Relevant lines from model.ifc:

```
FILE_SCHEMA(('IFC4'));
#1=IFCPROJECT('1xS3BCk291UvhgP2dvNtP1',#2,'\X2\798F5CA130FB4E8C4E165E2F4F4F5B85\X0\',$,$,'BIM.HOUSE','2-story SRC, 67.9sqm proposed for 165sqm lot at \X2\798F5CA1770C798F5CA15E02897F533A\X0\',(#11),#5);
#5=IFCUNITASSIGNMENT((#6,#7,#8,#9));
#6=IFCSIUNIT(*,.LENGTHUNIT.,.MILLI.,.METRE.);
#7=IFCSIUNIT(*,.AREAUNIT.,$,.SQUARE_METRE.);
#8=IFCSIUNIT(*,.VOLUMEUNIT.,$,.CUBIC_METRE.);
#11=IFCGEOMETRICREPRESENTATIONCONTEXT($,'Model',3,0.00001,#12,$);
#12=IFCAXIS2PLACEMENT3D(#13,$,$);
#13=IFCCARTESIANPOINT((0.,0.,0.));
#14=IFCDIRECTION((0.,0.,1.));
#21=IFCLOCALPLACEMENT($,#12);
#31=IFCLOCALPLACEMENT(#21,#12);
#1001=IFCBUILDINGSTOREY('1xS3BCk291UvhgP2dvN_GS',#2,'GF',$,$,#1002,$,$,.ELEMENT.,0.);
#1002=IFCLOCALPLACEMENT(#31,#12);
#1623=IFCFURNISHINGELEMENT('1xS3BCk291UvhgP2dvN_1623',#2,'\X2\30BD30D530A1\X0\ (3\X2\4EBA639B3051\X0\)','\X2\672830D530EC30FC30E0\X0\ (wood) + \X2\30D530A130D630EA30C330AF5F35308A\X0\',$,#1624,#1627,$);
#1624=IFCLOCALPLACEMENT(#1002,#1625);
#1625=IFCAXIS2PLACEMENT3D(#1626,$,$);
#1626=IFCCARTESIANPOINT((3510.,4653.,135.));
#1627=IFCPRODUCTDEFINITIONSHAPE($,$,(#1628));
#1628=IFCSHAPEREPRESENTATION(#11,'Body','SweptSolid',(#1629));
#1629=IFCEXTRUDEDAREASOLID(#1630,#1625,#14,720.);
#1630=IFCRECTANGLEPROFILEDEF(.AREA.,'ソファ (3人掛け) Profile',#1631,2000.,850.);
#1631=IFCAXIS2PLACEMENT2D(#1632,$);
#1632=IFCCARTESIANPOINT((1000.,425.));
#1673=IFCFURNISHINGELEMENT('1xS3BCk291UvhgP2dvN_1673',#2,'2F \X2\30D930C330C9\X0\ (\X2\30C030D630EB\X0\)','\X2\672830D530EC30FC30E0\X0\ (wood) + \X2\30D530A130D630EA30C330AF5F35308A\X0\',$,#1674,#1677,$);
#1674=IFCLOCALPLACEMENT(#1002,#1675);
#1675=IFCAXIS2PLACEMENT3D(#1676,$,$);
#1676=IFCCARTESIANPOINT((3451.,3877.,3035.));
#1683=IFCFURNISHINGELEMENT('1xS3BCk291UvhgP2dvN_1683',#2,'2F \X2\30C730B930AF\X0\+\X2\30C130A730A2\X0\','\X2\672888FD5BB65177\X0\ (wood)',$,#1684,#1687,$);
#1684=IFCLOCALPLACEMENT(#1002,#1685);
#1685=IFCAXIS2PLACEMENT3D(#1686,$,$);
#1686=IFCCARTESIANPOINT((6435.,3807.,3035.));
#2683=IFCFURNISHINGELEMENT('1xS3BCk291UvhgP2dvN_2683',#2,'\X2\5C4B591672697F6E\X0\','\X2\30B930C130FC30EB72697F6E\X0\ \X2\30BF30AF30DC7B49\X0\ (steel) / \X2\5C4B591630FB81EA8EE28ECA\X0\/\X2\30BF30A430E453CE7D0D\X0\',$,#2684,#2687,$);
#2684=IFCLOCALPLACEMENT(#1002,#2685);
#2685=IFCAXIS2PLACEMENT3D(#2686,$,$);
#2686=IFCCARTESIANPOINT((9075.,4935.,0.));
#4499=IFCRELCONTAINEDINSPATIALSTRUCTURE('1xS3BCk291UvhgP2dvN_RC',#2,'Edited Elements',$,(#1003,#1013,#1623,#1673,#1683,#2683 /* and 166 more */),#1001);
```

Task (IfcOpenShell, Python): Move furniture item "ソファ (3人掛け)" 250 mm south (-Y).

```python
import ifcopenshell
import ifcopenshell.api.geometry
import ifcopenshell.util.placement
import ifcopenshell.util.unit

model = ifcopenshell.open("model.ifc")
unit_scale = ifcopenshell.util.unit.calculate_unit_scale(model)

item = model.by_id(1623)
matrix = ifcopenshell.util.placement.get_local_placement(item.ObjectPlacement)
matrix[1, 3] -= 0.25 / unit_scale
ifcopenshell.api.geometry.edit_object_placement(model, product=item, matrix=matrix, is_si=False)

print(ifcopenshell.util.placement.get_local_placement(item.ObjectPlacement).round(3) + 0.0)

model.write("model_edited.ifc")
```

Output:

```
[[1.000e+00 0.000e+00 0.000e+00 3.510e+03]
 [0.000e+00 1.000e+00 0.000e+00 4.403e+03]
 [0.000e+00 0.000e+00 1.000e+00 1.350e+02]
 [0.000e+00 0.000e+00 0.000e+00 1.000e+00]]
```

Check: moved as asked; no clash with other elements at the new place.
